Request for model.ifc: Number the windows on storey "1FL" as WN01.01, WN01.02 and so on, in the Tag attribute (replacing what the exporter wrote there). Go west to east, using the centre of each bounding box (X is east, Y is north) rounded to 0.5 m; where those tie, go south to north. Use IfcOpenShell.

First a look at what the model holds.

```python
import ifcopenshell
import ifcopenshell.util.element
import ifcopenshell.util.placement

model = ifcopenshell.open("model.ifc")
print(model.schema)
storey = next(s for s in model.by_type("IfcBuildingStorey") if s.Name == "1FL")
windows = [e for e in ifcopenshell.util.element.get_decomposition(storey) if e.is_a("IfcWindow")]
for e in sorted(windows, key=lambda e: e.id()):
    origin = ifcopenshell.util.placement.get_local_placement(e.ObjectPlacement)[:3, 3]
    print(e.id(), e.Tag, e.Name, origin.round(2) + 0.0, sep=" | ")
```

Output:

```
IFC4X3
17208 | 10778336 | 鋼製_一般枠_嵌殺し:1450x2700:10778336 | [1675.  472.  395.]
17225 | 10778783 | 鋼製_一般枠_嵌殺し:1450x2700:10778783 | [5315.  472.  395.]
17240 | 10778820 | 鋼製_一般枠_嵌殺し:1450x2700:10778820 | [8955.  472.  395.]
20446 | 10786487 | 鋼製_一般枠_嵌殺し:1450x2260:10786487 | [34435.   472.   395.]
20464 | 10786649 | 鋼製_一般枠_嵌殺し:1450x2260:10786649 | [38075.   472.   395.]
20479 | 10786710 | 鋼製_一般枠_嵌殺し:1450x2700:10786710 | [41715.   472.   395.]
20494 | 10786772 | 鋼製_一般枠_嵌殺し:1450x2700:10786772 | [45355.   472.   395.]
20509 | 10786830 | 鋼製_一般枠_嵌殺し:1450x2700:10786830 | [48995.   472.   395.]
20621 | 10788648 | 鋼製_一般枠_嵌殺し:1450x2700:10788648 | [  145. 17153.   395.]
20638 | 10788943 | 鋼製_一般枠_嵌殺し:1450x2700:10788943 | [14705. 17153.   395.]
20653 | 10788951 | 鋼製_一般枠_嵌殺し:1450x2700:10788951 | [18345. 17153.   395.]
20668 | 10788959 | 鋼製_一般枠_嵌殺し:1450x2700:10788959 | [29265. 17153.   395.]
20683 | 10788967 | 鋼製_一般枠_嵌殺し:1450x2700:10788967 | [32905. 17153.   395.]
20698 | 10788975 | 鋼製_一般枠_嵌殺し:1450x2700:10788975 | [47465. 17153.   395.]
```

```python
import ifcopenshell
import ifcopenshell.geom
import ifcopenshell.util.element
import ifcopenshell.util.shape

model = ifcopenshell.open("model.ifc")
settings = ifcopenshell.geom.settings()
settings.set("use-world-coords", True)


def centre(element):
    shape = ifcopenshell.geom.create_shape(settings, element)
    return ifcopenshell.util.shape.get_bbox_centroid(shape.geometry)


storey = next(s for s in model.by_type("IfcBuildingStorey") if s.Name == "1FL")
windows = [e for e in ifcopenshell.util.element.get_decomposition(storey) if e.is_a("IfcWindow")]

# Insertion points can sit at a corner or the storey origin, so sort by the geometry (in metres).
centres = {e: centre(e) for e in windows}
windows.sort(key=lambda e: (round(centres[e][0] / 0.5), centres[e][1]))

for i, e in enumerate(windows, start=1):
    number = f"WN01.{i:02d}"
    e.Tag = number
    print(e.id(), number)

model.write("model_rev.ifc")
```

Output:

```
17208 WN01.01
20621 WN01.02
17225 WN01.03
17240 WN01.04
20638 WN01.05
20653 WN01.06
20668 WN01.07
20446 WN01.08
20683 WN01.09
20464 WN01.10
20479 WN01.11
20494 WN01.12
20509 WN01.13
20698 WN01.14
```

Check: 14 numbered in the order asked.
